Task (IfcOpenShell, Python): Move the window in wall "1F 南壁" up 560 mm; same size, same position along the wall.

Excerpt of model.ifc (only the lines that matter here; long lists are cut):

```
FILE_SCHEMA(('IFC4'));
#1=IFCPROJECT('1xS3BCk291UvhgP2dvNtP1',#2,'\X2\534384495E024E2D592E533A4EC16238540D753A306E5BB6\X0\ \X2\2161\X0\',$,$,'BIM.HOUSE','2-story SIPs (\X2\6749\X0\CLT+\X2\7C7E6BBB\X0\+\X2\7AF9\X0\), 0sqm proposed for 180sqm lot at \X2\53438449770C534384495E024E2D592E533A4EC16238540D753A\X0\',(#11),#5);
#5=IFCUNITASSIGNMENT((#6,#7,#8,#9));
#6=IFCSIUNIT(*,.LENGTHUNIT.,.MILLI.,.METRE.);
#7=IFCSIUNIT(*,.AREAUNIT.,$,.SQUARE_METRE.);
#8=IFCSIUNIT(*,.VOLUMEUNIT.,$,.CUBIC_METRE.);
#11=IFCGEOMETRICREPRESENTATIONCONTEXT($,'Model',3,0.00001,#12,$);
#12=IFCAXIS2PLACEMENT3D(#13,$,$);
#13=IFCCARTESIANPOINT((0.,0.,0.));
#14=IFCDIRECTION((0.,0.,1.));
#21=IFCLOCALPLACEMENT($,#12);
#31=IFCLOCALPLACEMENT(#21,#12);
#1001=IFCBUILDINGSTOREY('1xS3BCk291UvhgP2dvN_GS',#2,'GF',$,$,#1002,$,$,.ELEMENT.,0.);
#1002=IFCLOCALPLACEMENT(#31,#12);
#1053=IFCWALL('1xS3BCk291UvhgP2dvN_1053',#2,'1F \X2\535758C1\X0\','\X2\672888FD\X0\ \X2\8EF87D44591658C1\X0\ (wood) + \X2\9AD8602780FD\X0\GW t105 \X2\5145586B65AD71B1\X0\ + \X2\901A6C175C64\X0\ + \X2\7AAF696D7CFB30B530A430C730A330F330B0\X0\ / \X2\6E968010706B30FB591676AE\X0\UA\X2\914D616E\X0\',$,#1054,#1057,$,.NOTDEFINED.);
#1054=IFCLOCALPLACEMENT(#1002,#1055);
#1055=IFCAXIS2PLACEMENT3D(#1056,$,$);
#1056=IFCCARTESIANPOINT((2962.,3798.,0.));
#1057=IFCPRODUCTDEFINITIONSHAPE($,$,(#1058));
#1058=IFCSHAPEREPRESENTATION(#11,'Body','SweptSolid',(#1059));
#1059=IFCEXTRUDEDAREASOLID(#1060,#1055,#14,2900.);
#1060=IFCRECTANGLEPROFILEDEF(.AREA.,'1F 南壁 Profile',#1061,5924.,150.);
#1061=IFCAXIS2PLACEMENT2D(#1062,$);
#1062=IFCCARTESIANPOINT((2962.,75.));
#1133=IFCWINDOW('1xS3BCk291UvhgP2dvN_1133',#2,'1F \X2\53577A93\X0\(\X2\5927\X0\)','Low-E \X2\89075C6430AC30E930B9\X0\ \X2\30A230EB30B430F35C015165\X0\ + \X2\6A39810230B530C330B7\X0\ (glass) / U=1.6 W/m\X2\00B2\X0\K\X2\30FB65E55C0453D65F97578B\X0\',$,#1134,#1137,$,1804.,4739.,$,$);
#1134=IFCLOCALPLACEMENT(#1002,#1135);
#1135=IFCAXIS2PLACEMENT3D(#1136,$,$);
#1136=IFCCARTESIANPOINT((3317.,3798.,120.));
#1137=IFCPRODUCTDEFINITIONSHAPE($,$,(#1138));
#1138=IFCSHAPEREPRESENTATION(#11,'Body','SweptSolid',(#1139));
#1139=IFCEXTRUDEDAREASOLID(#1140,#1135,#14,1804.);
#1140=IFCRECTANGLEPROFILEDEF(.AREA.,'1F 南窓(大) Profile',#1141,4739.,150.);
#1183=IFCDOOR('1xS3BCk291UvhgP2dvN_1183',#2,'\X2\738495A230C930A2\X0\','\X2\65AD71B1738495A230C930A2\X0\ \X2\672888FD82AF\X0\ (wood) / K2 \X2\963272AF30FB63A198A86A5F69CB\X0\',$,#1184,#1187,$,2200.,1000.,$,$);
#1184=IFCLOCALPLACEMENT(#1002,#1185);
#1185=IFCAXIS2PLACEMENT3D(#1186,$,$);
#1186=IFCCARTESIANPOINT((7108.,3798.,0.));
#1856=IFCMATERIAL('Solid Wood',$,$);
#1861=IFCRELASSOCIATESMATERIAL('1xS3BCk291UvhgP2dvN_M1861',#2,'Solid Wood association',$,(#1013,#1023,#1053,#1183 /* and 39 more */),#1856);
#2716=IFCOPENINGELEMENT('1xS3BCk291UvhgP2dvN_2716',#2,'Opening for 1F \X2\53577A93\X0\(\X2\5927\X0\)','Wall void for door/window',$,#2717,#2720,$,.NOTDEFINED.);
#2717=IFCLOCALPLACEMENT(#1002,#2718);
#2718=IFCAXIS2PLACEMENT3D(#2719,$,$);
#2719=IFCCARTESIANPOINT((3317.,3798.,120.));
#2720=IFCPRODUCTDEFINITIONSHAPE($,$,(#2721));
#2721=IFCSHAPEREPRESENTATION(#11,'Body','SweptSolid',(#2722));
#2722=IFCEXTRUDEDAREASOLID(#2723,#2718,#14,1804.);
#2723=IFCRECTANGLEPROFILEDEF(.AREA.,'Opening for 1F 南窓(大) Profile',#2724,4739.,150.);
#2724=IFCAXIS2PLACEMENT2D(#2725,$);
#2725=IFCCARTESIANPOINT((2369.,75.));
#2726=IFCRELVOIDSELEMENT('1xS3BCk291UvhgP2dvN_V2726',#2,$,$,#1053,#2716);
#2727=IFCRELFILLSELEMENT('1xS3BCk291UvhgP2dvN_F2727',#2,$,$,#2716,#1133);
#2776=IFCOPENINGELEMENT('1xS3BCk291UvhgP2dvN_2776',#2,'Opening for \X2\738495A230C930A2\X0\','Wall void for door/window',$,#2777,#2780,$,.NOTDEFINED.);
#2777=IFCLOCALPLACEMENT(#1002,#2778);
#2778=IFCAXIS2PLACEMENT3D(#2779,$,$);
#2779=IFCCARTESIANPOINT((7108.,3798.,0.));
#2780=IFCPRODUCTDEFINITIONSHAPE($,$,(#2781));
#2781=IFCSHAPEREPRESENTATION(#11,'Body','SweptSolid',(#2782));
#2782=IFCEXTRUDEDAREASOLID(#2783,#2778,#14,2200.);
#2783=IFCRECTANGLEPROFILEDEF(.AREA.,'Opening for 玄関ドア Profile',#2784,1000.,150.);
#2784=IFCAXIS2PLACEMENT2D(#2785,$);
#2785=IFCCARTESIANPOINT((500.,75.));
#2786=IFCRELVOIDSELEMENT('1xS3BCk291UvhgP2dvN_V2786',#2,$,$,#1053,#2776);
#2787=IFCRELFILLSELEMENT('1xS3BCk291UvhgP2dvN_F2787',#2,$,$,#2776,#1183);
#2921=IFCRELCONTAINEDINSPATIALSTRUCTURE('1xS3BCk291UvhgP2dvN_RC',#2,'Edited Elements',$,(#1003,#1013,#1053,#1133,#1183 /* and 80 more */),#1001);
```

```python
import numpy as np
import ifcopenshell
import ifcopenshell.api.geometry
import ifcopenshell.util.placement
import ifcopenshell.util.unit

model = ifcopenshell.open("model.ifc")
unit_scale = ifcopenshell.util.unit.calculate_unit_scale(model)

window = model.by_guid("1xS3BCk291UvhgP2dvN_1133")
opening = window.FillsVoids[0].RelatingOpeningElement
dz = 0.56 / unit_scale

shift = np.array([0.0, 0.0, dz])
# The window is not placed relative to its opening, so move both.
for product in (opening, window):
    matrix = ifcopenshell.util.placement.get_local_placement(product.ObjectPlacement)
    matrix[:3, 3] += shift
    ifcopenshell.api.geometry.edit_object_placement(model, product=product, matrix=matrix, is_si=False)

print(f"moved by {dz * unit_scale:+.3f} m")

model.write("model_edited.ifc")
```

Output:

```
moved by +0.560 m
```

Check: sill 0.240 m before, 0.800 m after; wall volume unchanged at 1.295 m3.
